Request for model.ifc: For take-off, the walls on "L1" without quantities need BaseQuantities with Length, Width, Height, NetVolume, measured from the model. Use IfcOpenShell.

First a look at what the model holds.

```python
import ifcopenshell
import ifcopenshell.util.element
import ifcopenshell.util.unit

model = ifcopenshell.open("model.ifc")
print(model.schema)
for unit_type in ("LENGTHUNIT", "AREAUNIT", "VOLUMEUNIT"):
    print(unit_type, ifcopenshell.util.unit.calculate_unit_scale(model, unit_type))
storey = next(s for s in model.by_type("IfcBuildingStorey") if s.Name == "L1")
walls = [e for e in ifcopenshell.util.element.get_decomposition(storey) if e.is_a("IfcWall")]
for e in sorted(walls, key=lambda e: e.id()):
    print(e.id(), e.is_a(), e.Name, list(ifcopenshell.util.element.get_psets(e, qtos_only=True)), sep=" | ")
```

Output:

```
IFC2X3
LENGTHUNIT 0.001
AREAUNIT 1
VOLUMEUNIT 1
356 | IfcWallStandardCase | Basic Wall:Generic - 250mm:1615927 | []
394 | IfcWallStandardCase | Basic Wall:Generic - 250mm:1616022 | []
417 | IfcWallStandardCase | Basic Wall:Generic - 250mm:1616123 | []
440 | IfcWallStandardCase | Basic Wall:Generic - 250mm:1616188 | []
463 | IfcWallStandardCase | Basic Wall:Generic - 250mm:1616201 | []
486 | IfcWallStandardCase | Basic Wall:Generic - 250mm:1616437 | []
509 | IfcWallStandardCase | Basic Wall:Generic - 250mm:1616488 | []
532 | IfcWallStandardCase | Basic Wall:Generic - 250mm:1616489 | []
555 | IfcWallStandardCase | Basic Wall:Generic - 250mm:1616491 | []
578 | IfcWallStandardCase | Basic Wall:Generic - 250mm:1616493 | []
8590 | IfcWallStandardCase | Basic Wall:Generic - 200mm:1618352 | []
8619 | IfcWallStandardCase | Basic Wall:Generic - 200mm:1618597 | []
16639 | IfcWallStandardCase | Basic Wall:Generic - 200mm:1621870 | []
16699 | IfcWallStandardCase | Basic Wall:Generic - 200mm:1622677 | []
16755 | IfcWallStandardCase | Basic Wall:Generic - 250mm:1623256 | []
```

```python
import ifcopenshell
import ifcopenshell.api.pset
import ifcopenshell.geom
import ifcopenshell.util.element
import ifcopenshell.util.shape
import ifcopenshell.util.unit

model = ifcopenshell.open("model.ifc")
unit_scale = ifcopenshell.util.unit.calculate_unit_scale(model)
volume_scale = ifcopenshell.util.unit.calculate_unit_scale(model, "VOLUMEUNIT")
settings = ifcopenshell.geom.settings()

storey = next(s for s in model.by_type("IfcBuildingStorey") if s.Name == "L1")
walls = [e for e in ifcopenshell.util.element.get_decomposition(storey) if e.is_a("IfcWall")]

for e in sorted(walls, key=lambda e: e.id()):
    if ifcopenshell.util.element.get_psets(e, qtos_only=True, should_inherit=False):
        continue
    # Geometry comes back in metres, in the element's own axes.
    shape = ifcopenshell.geom.create_shape(settings, e)
    values = {
        "Length": ifcopenshell.util.shape.get_x(shape.geometry) / unit_scale,
        "Width": ifcopenshell.util.shape.get_y(shape.geometry) / unit_scale,
        "Height": ifcopenshell.util.shape.get_z(shape.geometry) / unit_scale,
        "NetVolume": ifcopenshell.util.shape.get_volume(shape.geometry) / volume_scale,
    }
    qto = ifcopenshell.api.pset.add_qto(model, product=e, name="BaseQuantities")
    ifcopenshell.api.pset.edit_qto(model, qto=qto, properties=values)
    print(e.id(), {k: round(v, 3) for k, v in values.items()})

model.write("model_updated.ifc")
```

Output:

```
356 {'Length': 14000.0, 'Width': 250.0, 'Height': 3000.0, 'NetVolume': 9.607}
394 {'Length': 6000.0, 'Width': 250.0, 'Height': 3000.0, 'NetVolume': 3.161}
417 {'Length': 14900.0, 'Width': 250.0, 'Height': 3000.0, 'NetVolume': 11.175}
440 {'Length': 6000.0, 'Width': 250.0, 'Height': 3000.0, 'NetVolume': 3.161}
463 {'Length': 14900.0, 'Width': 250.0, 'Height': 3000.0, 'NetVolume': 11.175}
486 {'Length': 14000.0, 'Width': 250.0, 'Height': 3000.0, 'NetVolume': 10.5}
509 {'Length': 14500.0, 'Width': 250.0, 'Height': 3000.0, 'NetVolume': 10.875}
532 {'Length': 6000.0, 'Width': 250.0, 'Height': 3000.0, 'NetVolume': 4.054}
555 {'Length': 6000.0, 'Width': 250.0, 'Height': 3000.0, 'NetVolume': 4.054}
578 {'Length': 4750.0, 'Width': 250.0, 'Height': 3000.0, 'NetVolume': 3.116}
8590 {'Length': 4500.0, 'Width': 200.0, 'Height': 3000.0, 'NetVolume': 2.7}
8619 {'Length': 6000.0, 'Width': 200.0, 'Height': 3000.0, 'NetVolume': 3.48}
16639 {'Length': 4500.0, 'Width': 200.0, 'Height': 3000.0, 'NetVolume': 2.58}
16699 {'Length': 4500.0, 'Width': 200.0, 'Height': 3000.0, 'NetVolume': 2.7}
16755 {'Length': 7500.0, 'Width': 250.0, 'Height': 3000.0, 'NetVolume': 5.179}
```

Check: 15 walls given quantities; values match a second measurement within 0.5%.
